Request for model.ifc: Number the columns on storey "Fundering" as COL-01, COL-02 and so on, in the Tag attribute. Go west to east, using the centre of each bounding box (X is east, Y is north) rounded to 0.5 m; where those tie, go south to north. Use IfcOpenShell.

First a look at what the model holds.

```python
import ifcopenshell
import ifcopenshell.util.element
import ifcopenshell.util.placement

model = ifcopenshell.open("model.ifc")
print(model.schema)
storey = next(s for s in model.by_type("IfcBuildingStorey") if s.Name == "Fundering")
columns = [e for e in ifcopenshell.util.element.get_decomposition(storey) if e.is_a("IfcColumn")]
for e in sorted(columns, key=lambda e: e.id()):
    origin = ifcopenshell.util.placement.get_local_placement(e.ObjectPlacement)[:3, 3]
    print(e.id(), e.Tag, e.Name, origin.round(2) + 0.0, sep=" | ")
```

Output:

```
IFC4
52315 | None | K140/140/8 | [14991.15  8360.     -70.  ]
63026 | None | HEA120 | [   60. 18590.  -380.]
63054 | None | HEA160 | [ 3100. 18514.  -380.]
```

```python
import ifcopenshell
import ifcopenshell.geom
import ifcopenshell.util.element
import ifcopenshell.util.shape

model = ifcopenshell.open("model.ifc")
settings = ifcopenshell.geom.settings()
settings.set("use-world-coords", True)


def centre(element):
    shape = ifcopenshell.geom.create_shape(settings, element)
    return ifcopenshell.util.shape.get_bbox_centroid(shape.geometry)


storey = next(s for s in model.by_type("IfcBuildingStorey") if s.Name == "Fundering")
columns = [e for e in ifcopenshell.util.element.get_decomposition(storey) if e.is_a("IfcColumn")]

# Insertion points can sit at a corner or the storey origin, so sort by the geometry (in metres).
centres = {e: centre(e) for e in columns}
columns.sort(key=lambda e: (round(centres[e][0] / 0.5), centres[e][1]))

for i, e in enumerate(columns, start=1):
    number = f"COL-{i:02d}"
    e.Tag = number
    print(e.id(), number)

model.write("model_v2.ifc")
```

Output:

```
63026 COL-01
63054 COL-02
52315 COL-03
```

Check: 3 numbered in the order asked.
